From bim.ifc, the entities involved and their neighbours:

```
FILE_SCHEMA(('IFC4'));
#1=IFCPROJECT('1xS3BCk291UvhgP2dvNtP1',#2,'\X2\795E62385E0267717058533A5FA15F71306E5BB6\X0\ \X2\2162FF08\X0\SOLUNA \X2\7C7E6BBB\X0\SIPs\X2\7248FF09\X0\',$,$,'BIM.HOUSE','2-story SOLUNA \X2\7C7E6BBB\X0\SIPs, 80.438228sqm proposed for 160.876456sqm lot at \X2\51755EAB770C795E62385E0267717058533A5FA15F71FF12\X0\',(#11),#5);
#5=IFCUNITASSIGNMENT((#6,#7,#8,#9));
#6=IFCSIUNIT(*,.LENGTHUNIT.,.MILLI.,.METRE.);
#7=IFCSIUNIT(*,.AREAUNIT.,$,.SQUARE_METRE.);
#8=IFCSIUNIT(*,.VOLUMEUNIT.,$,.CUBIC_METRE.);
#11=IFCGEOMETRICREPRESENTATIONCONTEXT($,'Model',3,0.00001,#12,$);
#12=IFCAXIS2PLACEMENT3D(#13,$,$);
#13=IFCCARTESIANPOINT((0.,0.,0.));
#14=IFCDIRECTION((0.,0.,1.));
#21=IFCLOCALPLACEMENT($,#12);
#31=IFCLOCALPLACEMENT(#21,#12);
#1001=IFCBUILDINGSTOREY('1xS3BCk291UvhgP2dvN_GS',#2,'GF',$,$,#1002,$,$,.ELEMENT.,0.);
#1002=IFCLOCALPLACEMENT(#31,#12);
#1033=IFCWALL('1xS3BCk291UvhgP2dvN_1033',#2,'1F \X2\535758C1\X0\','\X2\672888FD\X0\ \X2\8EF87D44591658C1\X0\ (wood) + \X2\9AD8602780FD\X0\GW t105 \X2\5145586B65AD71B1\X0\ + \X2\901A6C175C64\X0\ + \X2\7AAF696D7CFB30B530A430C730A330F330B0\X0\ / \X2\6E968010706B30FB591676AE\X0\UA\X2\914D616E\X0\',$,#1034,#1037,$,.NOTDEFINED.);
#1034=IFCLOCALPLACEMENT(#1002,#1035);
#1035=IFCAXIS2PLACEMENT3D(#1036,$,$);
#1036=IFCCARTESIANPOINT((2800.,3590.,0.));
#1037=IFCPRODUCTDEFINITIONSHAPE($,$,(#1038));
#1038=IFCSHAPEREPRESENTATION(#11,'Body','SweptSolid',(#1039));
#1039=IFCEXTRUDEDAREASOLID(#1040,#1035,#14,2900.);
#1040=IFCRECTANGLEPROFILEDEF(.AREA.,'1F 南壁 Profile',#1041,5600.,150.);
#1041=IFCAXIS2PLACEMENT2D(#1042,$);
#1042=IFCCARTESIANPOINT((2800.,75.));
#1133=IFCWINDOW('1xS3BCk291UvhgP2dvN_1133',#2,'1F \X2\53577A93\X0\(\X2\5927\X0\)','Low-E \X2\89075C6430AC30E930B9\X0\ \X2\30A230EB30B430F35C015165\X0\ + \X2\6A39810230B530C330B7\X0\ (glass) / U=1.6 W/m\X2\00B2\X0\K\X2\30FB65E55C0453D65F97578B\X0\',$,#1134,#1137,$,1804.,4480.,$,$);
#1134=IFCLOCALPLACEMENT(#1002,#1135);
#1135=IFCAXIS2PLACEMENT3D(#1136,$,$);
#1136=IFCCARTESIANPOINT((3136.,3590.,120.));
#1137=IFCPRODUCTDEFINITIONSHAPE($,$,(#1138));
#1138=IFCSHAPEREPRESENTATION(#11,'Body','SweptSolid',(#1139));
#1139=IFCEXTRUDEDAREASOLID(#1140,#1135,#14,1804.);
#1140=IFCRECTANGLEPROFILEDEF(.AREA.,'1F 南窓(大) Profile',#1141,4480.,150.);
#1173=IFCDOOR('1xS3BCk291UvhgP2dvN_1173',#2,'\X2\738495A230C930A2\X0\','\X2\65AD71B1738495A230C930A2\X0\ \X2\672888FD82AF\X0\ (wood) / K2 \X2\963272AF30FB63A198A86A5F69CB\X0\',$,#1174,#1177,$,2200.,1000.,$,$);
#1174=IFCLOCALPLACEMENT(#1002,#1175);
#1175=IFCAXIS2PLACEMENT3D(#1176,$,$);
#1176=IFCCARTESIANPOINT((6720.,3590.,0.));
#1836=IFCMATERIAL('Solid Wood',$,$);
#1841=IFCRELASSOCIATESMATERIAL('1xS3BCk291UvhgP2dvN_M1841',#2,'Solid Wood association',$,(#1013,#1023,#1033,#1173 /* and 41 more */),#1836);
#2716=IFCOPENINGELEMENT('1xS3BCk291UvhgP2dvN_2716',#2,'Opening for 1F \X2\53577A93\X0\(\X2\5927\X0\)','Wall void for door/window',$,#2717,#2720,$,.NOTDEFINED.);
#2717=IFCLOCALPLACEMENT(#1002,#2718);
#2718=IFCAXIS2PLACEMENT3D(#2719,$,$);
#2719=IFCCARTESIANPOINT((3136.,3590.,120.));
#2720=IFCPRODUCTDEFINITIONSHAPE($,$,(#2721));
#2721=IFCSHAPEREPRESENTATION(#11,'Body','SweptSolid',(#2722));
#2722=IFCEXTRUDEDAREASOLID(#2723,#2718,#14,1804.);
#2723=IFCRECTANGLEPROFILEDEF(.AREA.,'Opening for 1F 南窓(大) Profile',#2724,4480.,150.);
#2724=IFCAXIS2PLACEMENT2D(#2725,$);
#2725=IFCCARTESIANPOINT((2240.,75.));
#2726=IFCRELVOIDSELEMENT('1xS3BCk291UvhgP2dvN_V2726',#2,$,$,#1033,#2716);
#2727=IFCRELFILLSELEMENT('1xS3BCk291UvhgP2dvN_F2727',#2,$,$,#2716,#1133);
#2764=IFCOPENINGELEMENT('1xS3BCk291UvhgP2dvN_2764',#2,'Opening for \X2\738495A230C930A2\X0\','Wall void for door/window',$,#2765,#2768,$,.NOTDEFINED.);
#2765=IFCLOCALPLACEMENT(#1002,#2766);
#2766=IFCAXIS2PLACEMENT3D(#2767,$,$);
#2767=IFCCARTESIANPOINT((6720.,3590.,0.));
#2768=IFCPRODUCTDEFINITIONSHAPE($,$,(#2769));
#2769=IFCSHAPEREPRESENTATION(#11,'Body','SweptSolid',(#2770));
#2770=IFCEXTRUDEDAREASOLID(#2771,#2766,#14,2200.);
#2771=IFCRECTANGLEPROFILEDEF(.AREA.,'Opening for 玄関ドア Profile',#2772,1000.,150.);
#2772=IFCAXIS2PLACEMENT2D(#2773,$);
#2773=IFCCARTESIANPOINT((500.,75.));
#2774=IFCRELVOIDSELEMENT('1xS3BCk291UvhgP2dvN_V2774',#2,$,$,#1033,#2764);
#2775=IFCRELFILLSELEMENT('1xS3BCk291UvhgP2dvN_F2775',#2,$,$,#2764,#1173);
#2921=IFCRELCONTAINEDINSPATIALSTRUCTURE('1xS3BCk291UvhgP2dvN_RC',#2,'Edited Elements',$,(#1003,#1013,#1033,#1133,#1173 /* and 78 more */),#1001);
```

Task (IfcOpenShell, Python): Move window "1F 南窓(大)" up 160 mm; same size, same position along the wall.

```python
import numpy as np
import ifcopenshell
import ifcopenshell.api.geometry
import ifcopenshell.util.placement
import ifcopenshell.util.unit

model = ifcopenshell.open("bim.ifc")
unit_scale = ifcopenshell.util.unit.calculate_unit_scale(model)

window = model.by_guid("1xS3BCk291UvhgP2dvN_1133")
opening = window.FillsVoids[0].RelatingOpeningElement
dz = 0.16 / unit_scale

shift = np.array([0.0, 0.0, dz])
# The window is not placed relative to its opening, so move both.
for product in (opening, window):
    matrix = ifcopenshell.util.placement.get_local_placement(product.ObjectPlacement)
    matrix[:3, 3] += shift
    ifcopenshell.api.geometry.edit_object_placement(model, product=product, matrix=matrix, is_si=False)

print(f"moved by {dz * unit_scale:+.3f} m")

model.write("bim_v2.ifc")
```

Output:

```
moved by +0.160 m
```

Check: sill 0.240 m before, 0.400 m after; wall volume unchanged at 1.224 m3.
